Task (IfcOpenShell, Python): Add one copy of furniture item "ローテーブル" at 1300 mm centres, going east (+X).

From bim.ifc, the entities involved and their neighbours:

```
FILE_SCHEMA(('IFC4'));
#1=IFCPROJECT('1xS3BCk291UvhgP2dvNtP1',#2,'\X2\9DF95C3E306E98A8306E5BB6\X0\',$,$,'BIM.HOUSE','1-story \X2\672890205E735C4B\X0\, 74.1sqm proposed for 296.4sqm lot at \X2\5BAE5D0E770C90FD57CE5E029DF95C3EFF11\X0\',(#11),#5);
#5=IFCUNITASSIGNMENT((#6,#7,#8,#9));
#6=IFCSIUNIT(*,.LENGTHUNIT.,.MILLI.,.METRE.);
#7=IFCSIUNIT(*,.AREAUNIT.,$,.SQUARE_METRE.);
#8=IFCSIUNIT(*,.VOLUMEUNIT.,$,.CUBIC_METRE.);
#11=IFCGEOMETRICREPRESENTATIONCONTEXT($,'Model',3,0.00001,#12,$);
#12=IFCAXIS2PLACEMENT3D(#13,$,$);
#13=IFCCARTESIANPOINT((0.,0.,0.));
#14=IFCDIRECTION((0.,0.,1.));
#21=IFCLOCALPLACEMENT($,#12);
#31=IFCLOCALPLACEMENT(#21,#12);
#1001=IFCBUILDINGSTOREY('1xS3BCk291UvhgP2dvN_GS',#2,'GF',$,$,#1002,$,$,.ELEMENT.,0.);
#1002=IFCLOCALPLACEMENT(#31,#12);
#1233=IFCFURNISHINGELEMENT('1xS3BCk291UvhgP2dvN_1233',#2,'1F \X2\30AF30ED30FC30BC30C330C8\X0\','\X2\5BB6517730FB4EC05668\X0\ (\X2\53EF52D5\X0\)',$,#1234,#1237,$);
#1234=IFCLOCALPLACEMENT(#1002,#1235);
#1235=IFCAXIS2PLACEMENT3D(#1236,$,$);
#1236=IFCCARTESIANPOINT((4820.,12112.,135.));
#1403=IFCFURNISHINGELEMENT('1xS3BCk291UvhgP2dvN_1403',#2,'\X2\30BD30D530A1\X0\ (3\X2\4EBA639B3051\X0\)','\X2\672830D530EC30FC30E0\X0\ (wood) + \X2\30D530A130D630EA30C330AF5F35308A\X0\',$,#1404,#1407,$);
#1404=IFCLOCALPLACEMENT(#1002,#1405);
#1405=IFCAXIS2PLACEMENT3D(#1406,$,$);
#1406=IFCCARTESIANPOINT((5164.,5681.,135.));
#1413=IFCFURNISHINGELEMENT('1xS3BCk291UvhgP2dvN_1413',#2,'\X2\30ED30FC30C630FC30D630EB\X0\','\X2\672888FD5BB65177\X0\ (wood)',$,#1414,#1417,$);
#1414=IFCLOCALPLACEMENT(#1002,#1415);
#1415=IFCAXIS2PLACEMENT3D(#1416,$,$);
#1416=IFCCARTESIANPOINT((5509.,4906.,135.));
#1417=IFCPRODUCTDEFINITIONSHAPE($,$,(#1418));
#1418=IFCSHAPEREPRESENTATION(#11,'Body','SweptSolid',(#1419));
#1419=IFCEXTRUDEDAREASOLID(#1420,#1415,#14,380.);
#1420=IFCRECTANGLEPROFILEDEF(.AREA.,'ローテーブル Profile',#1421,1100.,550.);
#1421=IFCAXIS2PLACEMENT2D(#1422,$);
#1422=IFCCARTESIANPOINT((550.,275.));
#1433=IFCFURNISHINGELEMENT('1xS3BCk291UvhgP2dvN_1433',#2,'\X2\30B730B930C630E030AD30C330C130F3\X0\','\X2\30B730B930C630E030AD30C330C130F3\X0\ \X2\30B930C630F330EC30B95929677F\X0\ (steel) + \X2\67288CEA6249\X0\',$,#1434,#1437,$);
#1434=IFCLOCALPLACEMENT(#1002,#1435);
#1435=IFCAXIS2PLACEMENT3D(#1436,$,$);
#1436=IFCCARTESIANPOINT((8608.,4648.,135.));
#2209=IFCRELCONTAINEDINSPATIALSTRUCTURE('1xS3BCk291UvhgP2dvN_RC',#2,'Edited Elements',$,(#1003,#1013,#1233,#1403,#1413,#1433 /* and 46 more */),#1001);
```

```python
import numpy as np
import ifcopenshell
import ifcopenshell.api.geometry
import ifcopenshell.api.root
import ifcopenshell.util.element
import ifcopenshell.util.placement
import ifcopenshell.util.unit

model = ifcopenshell.open("bim.ifc")
unit_scale = ifcopenshell.util.unit.calculate_unit_scale(model)


def reuse_history(source, copy):
    """copy_class also copies each property set's owner history, people and application; keep the originals."""
    for rel in copy.IsDefinedBy:
        if rel.is_a("IfcRelDefinesByProperties") and (history := rel.RelatingPropertyDefinition.OwnerHistory):
            rel.RelatingPropertyDefinition.OwnerHistory = source.OwnerHistory
            ifcopenshell.util.element.remove_deep2(model, history)


source = model.by_id(1413)
base = ifcopenshell.util.placement.get_local_placement(source.ObjectPlacement)
step = np.array([1.0, 0.0, 0.0]) * 1.3 / unit_scale

for i in range(1, 2):
    copy = ifcopenshell.api.root.copy_class(model, product=source)
    copy.Representation = ifcopenshell.util.element.copy_deep(
        model, source.Representation, exclude=["IfcGeometricRepresentationContext", "IfcRepresentationMap"]
    )
    reuse_history(source, copy)
    matrix = base.copy()
    matrix[:3, 3] += i * step
    print("added at", matrix[:3, 3].round(3) + 0.0)
    ifcopenshell.api.geometry.edit_object_placement(model, product=copy, matrix=matrix, is_si=False)

model.write("bim_v2.ifc")
```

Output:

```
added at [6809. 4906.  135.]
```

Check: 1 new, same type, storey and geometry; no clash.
